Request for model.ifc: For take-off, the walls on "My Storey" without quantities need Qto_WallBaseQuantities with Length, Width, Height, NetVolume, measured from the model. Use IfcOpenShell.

First a look at what the model holds.

```python
import ifcopenshell
import ifcopenshell.util.element
import ifcopenshell.util.unit

model = ifcopenshell.open("model.ifc")
print(model.schema)
for unit_type in ("LENGTHUNIT", "AREAUNIT", "VOLUMEUNIT"):
    print(unit_type, ifcopenshell.util.unit.calculate_unit_scale(model, unit_type))
storey = next(s for s in model.by_type("IfcBuildingStorey") if s.Name == "My Storey")
walls = [e for e in ifcopenshell.util.element.get_decomposition(storey) if e.is_a("IfcWall")]
for e in sorted(walls, key=lambda e: e.id()):
    print(e.id(), e.is_a(), e.Name, list(ifcopenshell.util.element.get_psets(e, qtos_only=True)), sep=" | ")
```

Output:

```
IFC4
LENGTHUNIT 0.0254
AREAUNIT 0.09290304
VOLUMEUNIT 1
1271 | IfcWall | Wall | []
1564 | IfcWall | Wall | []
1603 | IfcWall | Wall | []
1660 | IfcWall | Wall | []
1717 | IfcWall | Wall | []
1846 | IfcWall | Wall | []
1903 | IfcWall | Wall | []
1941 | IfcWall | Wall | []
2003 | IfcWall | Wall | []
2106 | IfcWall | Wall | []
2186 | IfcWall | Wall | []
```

```python
import ifcopenshell
import ifcopenshell.api.pset
import ifcopenshell.geom
import ifcopenshell.util.element
import ifcopenshell.util.shape
import ifcopenshell.util.unit

model = ifcopenshell.open("model.ifc")
unit_scale = ifcopenshell.util.unit.calculate_unit_scale(model)
volume_scale = ifcopenshell.util.unit.calculate_unit_scale(model, "VOLUMEUNIT")
settings = ifcopenshell.geom.settings()

storey = next(s for s in model.by_type("IfcBuildingStorey") if s.Name == "My Storey")
walls = [e for e in ifcopenshell.util.element.get_decomposition(storey) if e.is_a("IfcWall")]

for e in sorted(walls, key=lambda e: e.id()):
    if ifcopenshell.util.element.get_psets(e, qtos_only=True, should_inherit=False):
        continue
    # Geometry comes back in metres, in the element's own axes.
    shape = ifcopenshell.geom.create_shape(settings, e)
    values = {
        "Length": ifcopenshell.util.shape.get_x(shape.geometry) / unit_scale,
        "Width": ifcopenshell.util.shape.get_y(shape.geometry) / unit_scale,
        "Height": ifcopenshell.util.shape.get_z(shape.geometry) / unit_scale,
        "NetVolume": ifcopenshell.util.shape.get_volume(shape.geometry) / volume_scale,
    }
    qto = ifcopenshell.api.pset.add_qto(model, product=e, name="Qto_WallBaseQuantities")
    ifcopenshell.api.pset.edit_qto(model, qto=qto, properties=values)
    print(e.id(), {k: round(v, 3) for k, v in values.items()})

model.write("model_rev.ifc")
```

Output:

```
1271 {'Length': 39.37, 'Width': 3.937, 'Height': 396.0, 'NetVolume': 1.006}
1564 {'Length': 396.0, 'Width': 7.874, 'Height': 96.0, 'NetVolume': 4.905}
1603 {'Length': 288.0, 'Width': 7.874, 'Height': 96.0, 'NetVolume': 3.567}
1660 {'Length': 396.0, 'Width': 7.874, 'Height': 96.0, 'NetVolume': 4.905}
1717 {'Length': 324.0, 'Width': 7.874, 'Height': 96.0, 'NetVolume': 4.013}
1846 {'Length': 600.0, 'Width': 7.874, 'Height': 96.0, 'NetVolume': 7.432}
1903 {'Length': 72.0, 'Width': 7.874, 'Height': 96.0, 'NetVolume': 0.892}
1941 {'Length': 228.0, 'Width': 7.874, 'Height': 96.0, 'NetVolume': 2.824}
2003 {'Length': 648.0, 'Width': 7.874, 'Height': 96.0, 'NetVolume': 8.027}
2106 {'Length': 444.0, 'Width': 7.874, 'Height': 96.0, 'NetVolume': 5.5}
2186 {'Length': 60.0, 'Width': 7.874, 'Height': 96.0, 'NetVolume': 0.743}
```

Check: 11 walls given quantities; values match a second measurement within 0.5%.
